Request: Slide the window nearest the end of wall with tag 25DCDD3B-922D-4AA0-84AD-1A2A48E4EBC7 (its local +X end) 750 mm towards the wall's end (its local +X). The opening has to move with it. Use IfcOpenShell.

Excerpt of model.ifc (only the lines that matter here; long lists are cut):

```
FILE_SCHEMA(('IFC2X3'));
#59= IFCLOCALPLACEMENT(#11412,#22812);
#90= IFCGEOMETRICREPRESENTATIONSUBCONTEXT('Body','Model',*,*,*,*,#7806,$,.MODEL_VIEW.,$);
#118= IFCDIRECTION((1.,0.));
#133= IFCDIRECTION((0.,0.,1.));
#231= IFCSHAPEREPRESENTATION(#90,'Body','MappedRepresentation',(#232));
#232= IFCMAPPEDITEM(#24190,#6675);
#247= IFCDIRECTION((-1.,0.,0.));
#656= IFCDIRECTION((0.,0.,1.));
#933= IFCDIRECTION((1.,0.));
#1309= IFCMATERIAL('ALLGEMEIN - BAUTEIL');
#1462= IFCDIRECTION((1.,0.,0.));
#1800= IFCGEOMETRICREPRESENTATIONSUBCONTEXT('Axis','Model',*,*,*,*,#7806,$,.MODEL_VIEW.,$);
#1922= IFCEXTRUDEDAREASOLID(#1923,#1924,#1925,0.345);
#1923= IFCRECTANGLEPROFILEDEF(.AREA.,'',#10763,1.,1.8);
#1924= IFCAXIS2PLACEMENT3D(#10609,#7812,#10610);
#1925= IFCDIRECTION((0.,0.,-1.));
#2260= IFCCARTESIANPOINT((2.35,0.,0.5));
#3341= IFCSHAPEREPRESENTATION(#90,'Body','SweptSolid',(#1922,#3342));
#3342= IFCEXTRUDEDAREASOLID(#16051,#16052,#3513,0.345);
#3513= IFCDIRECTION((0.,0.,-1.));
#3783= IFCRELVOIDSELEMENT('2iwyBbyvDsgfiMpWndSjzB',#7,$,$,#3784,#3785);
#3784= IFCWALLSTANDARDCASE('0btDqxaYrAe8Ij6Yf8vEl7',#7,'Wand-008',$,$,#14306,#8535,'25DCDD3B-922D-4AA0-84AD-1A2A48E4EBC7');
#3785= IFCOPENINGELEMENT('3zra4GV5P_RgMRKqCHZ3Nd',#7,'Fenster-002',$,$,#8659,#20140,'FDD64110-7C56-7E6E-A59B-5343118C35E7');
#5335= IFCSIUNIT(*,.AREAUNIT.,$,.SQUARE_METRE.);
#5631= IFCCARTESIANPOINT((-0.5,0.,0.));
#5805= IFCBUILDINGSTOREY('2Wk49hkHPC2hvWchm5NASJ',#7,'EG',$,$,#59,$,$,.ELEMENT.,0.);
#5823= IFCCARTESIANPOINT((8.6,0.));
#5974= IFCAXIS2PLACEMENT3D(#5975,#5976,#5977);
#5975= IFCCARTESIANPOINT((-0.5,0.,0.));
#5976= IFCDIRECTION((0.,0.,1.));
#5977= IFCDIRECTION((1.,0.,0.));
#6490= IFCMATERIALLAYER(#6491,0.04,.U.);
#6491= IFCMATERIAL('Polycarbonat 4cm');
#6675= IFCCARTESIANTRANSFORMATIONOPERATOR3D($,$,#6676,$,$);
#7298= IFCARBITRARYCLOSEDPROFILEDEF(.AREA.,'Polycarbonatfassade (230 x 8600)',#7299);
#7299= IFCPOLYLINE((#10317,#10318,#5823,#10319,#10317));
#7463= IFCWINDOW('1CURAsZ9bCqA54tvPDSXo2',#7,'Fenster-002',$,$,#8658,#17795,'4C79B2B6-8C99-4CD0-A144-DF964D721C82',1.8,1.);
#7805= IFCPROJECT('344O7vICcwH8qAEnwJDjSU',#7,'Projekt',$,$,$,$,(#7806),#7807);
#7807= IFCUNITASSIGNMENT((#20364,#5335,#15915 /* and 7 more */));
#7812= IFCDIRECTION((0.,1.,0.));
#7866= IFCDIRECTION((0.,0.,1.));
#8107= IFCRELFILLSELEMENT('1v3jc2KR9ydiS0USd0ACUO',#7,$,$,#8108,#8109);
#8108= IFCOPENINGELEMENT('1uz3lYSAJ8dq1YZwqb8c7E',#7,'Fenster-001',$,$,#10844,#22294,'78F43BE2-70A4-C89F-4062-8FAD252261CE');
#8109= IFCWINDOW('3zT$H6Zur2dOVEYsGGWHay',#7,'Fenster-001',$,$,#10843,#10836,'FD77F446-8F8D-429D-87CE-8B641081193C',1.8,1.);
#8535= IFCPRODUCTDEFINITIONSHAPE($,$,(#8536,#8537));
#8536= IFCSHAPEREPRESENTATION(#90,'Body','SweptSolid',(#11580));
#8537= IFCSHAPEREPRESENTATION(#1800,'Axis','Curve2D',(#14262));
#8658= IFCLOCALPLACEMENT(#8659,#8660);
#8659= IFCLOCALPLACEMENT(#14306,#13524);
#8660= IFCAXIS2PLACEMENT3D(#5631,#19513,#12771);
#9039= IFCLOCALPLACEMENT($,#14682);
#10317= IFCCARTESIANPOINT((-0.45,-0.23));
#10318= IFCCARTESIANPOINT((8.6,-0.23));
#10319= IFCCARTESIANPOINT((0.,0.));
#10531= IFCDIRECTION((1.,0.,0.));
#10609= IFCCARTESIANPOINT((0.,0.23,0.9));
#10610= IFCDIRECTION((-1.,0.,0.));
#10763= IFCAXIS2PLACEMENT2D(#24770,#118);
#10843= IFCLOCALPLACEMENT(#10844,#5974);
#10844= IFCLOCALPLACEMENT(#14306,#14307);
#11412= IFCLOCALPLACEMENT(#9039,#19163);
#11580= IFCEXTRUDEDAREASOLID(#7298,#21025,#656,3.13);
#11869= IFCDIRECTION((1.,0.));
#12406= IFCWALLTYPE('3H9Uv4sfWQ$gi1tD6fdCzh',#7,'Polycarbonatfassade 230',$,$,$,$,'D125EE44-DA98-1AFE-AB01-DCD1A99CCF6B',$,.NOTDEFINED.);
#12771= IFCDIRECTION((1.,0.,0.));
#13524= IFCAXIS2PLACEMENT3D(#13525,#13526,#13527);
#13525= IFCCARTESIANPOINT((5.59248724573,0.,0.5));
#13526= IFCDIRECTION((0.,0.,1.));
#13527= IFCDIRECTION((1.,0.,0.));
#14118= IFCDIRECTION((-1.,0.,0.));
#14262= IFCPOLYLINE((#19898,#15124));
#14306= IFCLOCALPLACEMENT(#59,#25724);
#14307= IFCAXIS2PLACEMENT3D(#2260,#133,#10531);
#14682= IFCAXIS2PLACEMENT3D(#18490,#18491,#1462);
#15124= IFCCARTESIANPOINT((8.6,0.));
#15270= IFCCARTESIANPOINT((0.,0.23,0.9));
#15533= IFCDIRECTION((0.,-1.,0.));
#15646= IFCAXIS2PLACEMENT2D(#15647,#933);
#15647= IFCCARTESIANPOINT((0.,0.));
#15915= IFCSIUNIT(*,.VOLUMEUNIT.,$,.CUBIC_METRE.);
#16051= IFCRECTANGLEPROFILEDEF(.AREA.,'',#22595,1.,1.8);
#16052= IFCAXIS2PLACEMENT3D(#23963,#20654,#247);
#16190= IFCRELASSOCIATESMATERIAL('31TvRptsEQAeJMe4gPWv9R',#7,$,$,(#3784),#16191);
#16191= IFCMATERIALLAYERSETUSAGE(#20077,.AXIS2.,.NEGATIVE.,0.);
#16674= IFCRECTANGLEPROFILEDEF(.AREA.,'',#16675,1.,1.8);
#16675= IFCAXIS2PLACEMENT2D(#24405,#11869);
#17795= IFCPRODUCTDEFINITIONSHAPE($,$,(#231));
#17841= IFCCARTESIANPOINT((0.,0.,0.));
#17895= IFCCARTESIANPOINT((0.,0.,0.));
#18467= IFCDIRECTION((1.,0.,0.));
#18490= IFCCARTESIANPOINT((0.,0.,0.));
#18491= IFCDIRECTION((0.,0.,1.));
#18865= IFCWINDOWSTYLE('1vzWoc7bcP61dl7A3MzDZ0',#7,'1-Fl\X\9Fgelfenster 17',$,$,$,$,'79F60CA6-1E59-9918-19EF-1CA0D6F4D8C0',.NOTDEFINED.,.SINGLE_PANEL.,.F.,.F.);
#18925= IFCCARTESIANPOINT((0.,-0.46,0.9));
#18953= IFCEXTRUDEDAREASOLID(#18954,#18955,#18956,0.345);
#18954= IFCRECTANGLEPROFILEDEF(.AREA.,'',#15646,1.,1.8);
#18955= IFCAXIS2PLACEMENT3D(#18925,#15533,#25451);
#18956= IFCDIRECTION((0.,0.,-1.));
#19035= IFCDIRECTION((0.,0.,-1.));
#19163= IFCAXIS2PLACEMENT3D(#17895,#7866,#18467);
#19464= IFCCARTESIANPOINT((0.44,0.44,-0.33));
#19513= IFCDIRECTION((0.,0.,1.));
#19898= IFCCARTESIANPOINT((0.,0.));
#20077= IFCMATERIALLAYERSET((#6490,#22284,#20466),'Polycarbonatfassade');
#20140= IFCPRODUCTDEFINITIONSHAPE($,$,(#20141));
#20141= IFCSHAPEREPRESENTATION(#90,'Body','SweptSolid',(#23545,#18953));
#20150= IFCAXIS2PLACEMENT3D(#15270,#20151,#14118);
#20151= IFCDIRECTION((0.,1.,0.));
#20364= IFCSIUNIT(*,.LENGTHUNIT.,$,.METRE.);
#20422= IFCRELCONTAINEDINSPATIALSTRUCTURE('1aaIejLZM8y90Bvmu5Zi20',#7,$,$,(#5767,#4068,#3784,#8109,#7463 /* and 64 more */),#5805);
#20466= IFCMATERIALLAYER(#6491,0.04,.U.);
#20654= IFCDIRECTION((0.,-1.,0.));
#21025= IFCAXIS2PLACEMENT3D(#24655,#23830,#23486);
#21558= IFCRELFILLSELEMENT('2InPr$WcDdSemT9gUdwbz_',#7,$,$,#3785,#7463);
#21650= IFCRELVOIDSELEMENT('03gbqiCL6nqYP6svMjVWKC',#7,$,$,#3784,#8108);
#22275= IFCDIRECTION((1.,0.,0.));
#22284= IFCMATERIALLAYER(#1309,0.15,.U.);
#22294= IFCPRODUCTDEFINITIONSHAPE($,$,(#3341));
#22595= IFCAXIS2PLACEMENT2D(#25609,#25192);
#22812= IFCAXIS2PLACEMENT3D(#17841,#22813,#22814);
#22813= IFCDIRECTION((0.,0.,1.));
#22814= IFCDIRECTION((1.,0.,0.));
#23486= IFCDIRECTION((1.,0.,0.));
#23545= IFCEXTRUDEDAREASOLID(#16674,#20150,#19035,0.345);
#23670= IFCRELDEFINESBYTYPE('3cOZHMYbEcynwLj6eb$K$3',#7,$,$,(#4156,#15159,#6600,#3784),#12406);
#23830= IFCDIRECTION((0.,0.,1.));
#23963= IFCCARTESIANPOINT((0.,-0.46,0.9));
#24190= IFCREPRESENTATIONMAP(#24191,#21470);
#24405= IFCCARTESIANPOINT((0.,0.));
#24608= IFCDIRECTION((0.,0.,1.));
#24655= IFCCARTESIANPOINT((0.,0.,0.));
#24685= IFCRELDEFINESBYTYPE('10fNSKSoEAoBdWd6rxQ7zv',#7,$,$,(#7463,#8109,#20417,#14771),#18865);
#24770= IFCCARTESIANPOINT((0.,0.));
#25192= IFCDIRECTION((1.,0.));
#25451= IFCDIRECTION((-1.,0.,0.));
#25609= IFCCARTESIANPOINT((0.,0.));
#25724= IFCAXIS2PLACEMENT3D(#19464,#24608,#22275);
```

```python
import ifcopenshell
import ifcopenshell.api.geometry
import ifcopenshell.util.placement
import ifcopenshell.util.unit

model = ifcopenshell.open("model.ifc")
unit_scale = ifcopenshell.util.unit.calculate_unit_scale(model)

window = model.by_guid("1CURAsZ9bCqA54tvPDSXo2")
opening = window.FillsVoids[0].RelatingOpeningElement
wall = opening.VoidsElements[0].RelatingBuildingElement

wall_matrix = ifcopenshell.util.placement.get_local_placement(wall.ObjectPlacement)
shift = wall_matrix[:3, 0] * 0.75 / unit_scale
before = ifcopenshell.util.placement.get_local_placement(window.ObjectPlacement)[:3, 3].copy()

# The window is placed relative to its opening, so it follows when the opening moves.
matrix = ifcopenshell.util.placement.get_local_placement(opening.ObjectPlacement)
matrix[:3, 3] += shift
ifcopenshell.api.geometry.edit_object_placement(
    model, product=opening, matrix=matrix, is_si=False, should_transform_children=True
)

after = ifcopenshell.util.placement.get_local_placement(window.ObjectPlacement)[:3, 3]
print("window moved by", (after - before).round(3) + 0.0)

model.write("model-out.ifc")
```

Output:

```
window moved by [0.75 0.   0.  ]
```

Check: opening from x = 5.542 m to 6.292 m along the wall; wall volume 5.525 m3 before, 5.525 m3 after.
